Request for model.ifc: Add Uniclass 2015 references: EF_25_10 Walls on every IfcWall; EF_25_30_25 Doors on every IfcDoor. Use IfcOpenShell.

First a look at what the model holds.

```python
import ifcopenshell

model = ifcopenshell.open("model.ifc")
print(model.schema)
print("classifications:", [c.Name for c in model.by_type("IfcClassification")])
for ifc_class in ("IfcDoor", "IfcRoof", "IfcStair", "IfcWall", "IfcWindow"):
    print(ifc_class, len(model.by_type(ifc_class)))
```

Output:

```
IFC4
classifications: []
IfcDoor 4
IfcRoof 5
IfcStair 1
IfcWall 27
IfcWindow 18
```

```python
import ifcopenshell
import ifcopenshell.api.classification

model = ifcopenshell.open("model.ifc")

system = ifcopenshell.api.classification.add_classification(model, classification="Uniclass 2015")

codes = {
    "IfcWall": ("EF_25_10", "Walls"),
    "IfcDoor": ("EF_25_30_25", "Doors"),
}
for ifc_class, (code, name) in codes.items():
    products = model.by_type(ifc_class)
    ifcopenshell.api.classification.add_reference(
        model, products=products, classification=system, identification=code, name=name
    )
    print(code, len(products))

model.write("model-out.ifc")
```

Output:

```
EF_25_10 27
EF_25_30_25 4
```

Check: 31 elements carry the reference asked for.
